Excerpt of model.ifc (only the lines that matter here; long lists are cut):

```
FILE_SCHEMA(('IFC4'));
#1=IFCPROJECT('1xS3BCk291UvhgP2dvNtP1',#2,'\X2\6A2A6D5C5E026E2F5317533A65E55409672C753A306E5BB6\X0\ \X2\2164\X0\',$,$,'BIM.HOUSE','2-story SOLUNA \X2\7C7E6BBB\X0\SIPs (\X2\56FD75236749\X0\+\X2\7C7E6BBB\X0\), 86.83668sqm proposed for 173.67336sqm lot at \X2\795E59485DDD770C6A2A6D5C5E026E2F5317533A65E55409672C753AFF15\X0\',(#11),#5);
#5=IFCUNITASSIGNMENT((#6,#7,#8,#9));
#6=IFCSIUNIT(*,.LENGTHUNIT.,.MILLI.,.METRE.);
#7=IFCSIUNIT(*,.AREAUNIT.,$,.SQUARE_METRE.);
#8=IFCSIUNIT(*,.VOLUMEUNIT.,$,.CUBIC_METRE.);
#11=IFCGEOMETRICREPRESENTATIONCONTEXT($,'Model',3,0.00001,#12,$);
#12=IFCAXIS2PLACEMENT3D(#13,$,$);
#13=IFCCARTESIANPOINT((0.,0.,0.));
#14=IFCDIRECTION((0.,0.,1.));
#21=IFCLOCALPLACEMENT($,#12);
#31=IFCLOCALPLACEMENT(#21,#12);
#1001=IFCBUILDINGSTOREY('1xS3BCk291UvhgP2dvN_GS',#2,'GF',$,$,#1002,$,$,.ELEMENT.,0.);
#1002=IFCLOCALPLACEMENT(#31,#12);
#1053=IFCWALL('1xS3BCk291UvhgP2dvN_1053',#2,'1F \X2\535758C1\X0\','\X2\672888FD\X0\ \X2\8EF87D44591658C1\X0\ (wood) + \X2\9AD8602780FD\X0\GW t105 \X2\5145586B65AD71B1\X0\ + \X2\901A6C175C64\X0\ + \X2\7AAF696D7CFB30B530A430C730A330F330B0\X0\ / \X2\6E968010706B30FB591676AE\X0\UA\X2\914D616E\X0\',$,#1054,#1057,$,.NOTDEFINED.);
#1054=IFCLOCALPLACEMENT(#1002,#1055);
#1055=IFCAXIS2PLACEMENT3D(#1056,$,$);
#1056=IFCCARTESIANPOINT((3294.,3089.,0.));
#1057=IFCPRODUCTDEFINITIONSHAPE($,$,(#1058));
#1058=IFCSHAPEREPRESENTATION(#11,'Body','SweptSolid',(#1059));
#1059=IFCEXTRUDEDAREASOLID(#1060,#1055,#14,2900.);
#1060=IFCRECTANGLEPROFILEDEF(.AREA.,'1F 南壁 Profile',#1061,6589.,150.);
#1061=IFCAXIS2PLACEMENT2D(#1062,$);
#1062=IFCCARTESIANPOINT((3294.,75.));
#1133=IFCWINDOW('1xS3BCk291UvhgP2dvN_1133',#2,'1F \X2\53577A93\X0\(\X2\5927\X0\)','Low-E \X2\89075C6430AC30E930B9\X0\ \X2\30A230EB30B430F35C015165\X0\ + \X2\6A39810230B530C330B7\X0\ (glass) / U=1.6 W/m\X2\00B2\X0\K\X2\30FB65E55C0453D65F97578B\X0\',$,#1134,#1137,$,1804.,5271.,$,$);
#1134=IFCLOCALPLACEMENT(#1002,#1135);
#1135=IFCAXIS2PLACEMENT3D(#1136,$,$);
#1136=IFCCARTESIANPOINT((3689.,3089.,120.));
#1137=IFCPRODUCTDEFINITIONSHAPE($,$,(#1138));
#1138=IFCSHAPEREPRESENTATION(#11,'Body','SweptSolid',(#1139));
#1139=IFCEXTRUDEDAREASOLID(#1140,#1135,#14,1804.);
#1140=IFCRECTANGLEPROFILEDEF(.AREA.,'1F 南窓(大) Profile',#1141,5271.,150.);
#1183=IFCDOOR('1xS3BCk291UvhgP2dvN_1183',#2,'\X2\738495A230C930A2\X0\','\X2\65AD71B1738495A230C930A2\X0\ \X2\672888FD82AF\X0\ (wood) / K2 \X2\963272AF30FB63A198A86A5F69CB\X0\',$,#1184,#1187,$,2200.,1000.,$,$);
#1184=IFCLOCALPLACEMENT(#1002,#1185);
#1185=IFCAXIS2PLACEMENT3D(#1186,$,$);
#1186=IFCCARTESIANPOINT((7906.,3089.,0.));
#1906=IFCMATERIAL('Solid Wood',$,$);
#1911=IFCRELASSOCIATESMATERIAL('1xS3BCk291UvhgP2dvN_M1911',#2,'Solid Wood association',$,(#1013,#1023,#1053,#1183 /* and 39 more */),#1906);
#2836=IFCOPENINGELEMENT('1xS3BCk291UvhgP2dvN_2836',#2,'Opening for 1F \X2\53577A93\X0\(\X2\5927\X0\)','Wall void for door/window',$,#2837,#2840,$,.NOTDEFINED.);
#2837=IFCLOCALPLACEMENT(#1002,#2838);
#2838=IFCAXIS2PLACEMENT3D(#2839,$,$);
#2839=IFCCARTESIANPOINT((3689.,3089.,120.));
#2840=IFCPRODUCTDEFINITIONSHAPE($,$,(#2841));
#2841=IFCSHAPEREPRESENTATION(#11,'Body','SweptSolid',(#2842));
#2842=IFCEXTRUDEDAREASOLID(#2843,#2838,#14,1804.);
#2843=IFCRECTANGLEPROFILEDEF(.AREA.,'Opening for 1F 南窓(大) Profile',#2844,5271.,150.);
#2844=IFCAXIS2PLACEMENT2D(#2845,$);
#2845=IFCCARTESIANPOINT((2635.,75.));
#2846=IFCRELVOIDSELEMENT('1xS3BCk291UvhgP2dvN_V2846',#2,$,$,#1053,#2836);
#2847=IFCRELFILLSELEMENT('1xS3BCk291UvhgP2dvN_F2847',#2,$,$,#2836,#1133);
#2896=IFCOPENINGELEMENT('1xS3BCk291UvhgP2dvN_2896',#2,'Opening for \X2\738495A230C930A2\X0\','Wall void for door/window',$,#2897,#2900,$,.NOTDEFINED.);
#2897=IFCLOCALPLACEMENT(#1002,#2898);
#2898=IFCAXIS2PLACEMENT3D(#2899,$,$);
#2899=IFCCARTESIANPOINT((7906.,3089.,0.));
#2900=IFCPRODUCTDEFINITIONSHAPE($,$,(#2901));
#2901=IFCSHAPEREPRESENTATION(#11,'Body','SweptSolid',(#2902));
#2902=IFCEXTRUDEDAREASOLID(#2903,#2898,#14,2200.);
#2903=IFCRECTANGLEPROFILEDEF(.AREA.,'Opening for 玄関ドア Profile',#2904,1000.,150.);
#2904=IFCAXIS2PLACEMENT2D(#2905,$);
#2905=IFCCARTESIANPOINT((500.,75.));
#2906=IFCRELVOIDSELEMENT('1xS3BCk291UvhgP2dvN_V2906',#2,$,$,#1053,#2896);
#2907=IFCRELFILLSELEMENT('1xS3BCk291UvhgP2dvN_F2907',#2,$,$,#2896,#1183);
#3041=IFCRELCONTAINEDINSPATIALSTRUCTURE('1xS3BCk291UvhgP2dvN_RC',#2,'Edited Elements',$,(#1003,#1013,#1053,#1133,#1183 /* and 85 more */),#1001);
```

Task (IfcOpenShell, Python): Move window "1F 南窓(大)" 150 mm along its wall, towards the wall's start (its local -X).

```python
import ifcopenshell
import ifcopenshell.api.geometry
import ifcopenshell.util.placement
import ifcopenshell.util.unit

model = ifcopenshell.open("model.ifc")
unit_scale = ifcopenshell.util.unit.calculate_unit_scale(model)

window = model.by_guid("1xS3BCk291UvhgP2dvN_1133")
opening = window.FillsVoids[0].RelatingOpeningElement
wall = opening.VoidsElements[0].RelatingBuildingElement

wall_matrix = ifcopenshell.util.placement.get_local_placement(wall.ObjectPlacement)
shift = wall_matrix[:3, 0] * -0.15 / unit_scale
before = ifcopenshell.util.placement.get_local_placement(window.ObjectPlacement)[:3, 3].copy()

# The window is not placed relative to its opening, so move both.
for product in (opening, window):
    matrix = ifcopenshell.util.placement.get_local_placement(product.ObjectPlacement)
    matrix[:3, 3] += shift
    ifcopenshell.api.geometry.edit_object_placement(model, product=product, matrix=matrix, is_si=False)

after = ifcopenshell.util.placement.get_local_placement(window.ObjectPlacement)[:3, 3]
print("window moved by", (after - before).round(3) + 0.0)

model.write("model-out.ifc")
```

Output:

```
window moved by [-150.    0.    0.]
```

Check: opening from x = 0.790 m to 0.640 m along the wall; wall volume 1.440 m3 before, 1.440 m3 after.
